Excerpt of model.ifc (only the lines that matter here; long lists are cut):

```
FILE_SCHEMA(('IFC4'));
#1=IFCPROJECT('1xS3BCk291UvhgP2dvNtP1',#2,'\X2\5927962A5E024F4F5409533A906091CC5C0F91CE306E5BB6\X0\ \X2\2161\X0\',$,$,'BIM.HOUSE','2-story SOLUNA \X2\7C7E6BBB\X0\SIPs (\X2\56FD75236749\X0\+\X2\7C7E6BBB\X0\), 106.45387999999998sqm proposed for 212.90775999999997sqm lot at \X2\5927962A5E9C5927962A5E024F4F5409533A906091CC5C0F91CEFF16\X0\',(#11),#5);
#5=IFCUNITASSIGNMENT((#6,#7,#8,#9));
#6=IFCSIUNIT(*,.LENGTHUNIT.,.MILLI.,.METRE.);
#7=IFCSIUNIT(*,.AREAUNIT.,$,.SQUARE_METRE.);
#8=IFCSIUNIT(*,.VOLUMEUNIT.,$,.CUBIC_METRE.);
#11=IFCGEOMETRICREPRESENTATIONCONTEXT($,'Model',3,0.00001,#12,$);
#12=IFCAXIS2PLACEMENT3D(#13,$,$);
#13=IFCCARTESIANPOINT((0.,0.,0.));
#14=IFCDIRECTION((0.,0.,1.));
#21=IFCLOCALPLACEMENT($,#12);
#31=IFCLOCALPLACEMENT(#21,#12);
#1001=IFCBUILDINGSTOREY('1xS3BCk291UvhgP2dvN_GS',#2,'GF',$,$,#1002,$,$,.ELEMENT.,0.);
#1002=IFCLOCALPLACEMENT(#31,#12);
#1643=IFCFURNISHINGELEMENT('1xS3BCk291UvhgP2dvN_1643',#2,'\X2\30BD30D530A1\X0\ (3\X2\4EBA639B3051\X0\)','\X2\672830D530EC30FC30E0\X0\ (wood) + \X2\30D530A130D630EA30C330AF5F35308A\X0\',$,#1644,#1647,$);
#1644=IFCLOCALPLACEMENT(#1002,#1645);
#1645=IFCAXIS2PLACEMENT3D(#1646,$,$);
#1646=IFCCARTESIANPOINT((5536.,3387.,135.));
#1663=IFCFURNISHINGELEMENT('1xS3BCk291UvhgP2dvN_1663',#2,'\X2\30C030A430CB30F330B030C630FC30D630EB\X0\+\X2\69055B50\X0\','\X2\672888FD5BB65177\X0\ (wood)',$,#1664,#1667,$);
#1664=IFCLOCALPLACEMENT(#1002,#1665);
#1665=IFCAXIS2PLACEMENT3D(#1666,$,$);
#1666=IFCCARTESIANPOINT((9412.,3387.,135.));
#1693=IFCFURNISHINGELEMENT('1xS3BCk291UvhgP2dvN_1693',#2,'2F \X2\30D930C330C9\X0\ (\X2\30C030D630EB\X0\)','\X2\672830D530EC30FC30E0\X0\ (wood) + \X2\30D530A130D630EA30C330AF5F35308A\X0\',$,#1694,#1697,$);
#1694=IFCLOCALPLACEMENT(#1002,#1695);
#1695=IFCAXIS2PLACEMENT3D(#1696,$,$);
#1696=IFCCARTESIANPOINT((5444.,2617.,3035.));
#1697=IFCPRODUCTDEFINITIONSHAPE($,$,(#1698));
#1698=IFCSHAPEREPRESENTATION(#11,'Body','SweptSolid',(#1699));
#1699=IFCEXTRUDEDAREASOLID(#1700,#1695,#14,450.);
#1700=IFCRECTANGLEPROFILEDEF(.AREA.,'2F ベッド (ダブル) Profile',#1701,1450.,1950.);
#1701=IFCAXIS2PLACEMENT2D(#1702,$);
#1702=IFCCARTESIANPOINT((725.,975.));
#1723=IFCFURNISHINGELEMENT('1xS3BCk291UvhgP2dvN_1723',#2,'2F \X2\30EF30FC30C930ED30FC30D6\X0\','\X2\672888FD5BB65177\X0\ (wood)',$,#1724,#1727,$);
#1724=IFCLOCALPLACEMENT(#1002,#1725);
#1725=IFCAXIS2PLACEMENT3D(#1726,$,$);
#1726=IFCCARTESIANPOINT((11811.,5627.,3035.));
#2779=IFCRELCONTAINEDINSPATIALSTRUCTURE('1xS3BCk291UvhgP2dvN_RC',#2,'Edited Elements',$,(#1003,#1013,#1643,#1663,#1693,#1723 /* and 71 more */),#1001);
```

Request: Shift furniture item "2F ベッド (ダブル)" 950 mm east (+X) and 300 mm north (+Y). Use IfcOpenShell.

```python
import ifcopenshell
import ifcopenshell.api.geometry
import ifcopenshell.util.placement
import ifcopenshell.util.unit

model = ifcopenshell.open("model.ifc")
unit_scale = ifcopenshell.util.unit.calculate_unit_scale(model)

item = model.by_id(1693)
matrix = ifcopenshell.util.placement.get_local_placement(item.ObjectPlacement)
matrix[0, 3] += 0.95 / unit_scale
matrix[1, 3] += 0.3 / unit_scale
ifcopenshell.api.geometry.edit_object_placement(model, product=item, matrix=matrix, is_si=False)

print(ifcopenshell.util.placement.get_local_placement(item.ObjectPlacement).round(3) + 0.0)

model.write("model-out.ifc")
```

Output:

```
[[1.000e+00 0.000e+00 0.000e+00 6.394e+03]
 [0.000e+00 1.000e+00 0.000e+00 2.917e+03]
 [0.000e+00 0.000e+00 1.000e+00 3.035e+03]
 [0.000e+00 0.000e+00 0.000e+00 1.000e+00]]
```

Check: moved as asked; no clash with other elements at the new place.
